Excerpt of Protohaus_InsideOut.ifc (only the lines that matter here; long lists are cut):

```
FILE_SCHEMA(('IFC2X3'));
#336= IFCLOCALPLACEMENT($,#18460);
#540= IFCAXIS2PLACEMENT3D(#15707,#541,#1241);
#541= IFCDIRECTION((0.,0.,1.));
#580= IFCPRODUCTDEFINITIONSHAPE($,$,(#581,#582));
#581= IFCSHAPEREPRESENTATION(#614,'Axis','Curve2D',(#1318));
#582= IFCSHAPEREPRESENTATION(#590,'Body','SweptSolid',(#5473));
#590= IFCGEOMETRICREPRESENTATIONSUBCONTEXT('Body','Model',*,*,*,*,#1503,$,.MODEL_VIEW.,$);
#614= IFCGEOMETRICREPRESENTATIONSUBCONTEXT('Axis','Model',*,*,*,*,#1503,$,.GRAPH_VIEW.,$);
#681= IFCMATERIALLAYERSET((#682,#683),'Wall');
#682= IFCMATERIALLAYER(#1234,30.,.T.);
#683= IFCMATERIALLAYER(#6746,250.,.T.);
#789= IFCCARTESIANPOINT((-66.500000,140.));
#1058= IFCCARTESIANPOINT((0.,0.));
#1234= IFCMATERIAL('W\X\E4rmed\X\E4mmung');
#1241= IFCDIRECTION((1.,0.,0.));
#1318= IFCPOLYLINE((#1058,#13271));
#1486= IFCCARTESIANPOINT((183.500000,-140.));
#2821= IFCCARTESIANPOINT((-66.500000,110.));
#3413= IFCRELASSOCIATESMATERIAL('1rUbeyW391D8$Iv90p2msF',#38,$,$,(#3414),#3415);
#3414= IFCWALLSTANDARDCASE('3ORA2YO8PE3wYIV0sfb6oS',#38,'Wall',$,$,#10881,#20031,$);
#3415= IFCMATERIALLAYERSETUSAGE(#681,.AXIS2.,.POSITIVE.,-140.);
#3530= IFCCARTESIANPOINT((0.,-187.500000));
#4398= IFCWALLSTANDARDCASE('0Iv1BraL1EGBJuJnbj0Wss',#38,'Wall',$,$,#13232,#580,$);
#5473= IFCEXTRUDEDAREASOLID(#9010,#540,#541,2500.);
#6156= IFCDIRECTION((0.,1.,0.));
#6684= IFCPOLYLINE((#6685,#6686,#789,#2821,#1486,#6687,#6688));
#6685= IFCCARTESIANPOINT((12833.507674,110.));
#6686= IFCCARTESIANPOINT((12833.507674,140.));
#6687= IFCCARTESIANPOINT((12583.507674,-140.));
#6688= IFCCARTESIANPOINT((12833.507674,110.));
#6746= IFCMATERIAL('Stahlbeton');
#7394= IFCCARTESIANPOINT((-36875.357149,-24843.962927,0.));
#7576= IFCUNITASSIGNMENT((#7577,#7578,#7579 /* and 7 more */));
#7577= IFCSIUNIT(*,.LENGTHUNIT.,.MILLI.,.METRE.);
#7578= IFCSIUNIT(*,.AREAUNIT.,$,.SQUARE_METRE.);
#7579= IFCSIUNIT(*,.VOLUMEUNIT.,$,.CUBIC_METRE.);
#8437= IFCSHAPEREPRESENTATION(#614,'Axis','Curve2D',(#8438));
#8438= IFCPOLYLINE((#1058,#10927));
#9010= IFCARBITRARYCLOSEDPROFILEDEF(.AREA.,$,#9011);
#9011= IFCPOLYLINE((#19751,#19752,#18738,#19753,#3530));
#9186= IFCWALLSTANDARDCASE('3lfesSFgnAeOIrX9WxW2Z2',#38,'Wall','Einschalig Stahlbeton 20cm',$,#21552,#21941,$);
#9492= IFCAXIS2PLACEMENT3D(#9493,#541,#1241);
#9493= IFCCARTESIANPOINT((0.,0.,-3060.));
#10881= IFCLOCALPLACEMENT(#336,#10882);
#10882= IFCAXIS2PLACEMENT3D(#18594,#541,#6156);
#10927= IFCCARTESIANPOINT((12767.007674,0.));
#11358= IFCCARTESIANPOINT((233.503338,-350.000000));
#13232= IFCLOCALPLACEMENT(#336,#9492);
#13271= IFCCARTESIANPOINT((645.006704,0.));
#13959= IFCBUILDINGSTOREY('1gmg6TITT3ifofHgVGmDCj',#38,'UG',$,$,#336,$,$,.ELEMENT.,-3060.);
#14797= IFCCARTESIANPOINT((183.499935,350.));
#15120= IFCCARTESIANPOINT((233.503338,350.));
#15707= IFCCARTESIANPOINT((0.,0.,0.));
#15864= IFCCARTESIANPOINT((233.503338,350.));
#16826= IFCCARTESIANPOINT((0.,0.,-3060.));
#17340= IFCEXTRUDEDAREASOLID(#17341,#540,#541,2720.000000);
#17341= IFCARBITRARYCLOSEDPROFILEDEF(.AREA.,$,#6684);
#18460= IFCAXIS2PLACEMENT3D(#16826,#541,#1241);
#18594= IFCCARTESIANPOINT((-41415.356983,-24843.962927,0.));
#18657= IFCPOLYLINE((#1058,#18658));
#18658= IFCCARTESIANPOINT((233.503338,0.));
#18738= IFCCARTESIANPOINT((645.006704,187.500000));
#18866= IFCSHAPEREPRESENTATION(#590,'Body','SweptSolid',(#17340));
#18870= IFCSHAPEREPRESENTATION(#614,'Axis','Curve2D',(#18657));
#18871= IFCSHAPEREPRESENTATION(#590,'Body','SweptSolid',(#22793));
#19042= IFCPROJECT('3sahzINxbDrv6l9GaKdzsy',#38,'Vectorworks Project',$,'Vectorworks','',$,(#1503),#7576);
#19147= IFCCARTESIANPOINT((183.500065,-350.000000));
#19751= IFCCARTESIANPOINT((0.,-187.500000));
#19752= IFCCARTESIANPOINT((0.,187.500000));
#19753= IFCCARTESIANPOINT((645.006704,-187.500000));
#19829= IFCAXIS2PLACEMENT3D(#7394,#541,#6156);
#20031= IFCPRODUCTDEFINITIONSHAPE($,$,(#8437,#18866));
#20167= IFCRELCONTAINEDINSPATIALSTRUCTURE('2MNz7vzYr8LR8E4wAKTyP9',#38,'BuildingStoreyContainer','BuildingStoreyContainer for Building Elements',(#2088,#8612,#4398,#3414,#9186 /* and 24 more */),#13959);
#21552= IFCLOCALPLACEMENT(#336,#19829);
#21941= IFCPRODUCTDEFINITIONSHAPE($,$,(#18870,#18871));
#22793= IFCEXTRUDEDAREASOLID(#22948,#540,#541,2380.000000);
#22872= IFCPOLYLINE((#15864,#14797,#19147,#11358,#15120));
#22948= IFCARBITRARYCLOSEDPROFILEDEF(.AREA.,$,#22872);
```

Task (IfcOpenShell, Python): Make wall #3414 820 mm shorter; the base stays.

```python
import ifcopenshell
import ifcopenshell.geom
import ifcopenshell.util.representation
import ifcopenshell.util.shape
import ifcopenshell.util.unit

model = ifcopenshell.open("Protohaus_InsideOut.ifc")
unit_scale = ifcopenshell.util.unit.calculate_unit_scale(model)
settings = ifcopenshell.geom.settings()


def volume(element):
    """Net volume in cubic metres, openings subtracted."""
    shape = ifcopenshell.geom.create_shape(settings, element)
    return ifcopenshell.util.shape.get_volume(shape.geometry)


wall = model.by_guid("3ORA2YO8PE3wYIV0sfb6oS")
before = volume(wall)

body = ifcopenshell.util.representation.get_representation(wall, "Model", "Body")
solid = body.Items[0]
old_height = solid.Depth
solid.Depth -= 0.82 / unit_scale
after = volume(wall)

print(f"height {old_height:g} -> {solid.Depth:g}, volume {before:.3f} -> {after:.3f} m3")

model.write("Protohaus_InsideOut_updated.ifc")
```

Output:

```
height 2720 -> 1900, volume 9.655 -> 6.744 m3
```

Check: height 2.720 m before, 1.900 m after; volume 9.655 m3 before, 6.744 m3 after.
